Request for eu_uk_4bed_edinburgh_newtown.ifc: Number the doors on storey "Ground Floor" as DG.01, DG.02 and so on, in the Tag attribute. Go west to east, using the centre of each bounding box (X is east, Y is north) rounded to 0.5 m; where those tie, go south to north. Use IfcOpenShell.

First a look at what the model holds.

```python
import ifcopenshell
import ifcopenshell.util.element
import ifcopenshell.util.placement

model = ifcopenshell.open("eu_uk_4bed_edinburgh_newtown.ifc")
print(model.schema)
storey = next(s for s in model.by_type("IfcBuildingStorey") if s.Name == "Ground Floor")
doors = [e for e in ifcopenshell.util.element.get_decomposition(storey) if e.is_a("IfcDoor")]
for e in sorted(doors, key=lambda e: e.id()):
    origin = ifcopenshell.util.placement.get_local_placement(e.ObjectPlacement)[:3, 3]
    print(e.id(), e.Tag, e.Name, origin.round(2) + 0.0, sep=" | ")
```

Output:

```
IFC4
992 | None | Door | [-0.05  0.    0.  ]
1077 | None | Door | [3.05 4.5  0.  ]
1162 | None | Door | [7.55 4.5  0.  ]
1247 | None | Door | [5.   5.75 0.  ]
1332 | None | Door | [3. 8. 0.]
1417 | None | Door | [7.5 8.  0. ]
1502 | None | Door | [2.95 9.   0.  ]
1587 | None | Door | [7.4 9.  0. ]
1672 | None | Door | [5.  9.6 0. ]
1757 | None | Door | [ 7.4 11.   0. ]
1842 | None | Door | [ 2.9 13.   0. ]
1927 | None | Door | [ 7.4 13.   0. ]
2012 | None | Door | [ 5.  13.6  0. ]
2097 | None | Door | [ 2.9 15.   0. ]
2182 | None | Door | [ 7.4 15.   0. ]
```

```python
import ifcopenshell
import ifcopenshell.geom
import ifcopenshell.util.element
import ifcopenshell.util.shape

model = ifcopenshell.open("eu_uk_4bed_edinburgh_newtown.ifc")
settings = ifcopenshell.geom.settings()
settings.set("use-world-coords", True)


def centre(element):
    shape = ifcopenshell.geom.create_shape(settings, element)
    return ifcopenshell.util.shape.get_bbox_centroid(shape.geometry)


storey = next(s for s in model.by_type("IfcBuildingStorey") if s.Name == "Ground Floor")
doors = [e for e in ifcopenshell.util.element.get_decomposition(storey) if e.is_a("IfcDoor")]

# Insertion points can sit at a corner or the storey origin, so sort by the geometry (in metres).
centres = {e: centre(e) for e in doors}
doors.sort(key=lambda e: (round(centres[e][0] / 0.5), centres[e][1]))

for i, e in enumerate(doors, start=1):
    number = f"DG.{i:02d}"
    e.Tag = number
    print(e.id(), number)

model.write("eu_uk_4bed_edinburgh_newtown_rev.ifc")
```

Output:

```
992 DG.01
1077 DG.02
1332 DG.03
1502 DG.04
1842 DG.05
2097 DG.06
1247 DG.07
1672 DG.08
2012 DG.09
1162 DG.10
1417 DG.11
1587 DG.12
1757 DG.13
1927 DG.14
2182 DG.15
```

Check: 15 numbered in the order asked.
